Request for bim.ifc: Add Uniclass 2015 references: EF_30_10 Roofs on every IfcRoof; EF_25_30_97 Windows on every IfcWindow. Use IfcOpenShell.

First a look at what the model holds.

```python
import ifcopenshell

model = ifcopenshell.open("bim.ifc")
print(model.schema)
print("classifications:", [c.Name for c in model.by_type("IfcClassification")])
for ifc_class in ("IfcDoor", "IfcRoof", "IfcStair", "IfcWall", "IfcWindow"):
    print(ifc_class, len(model.by_type(ifc_class)))
```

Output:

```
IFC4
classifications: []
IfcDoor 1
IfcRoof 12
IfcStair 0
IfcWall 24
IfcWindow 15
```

```python
import ifcopenshell
import ifcopenshell.api.classification

model = ifcopenshell.open("bim.ifc")

system = ifcopenshell.api.classification.add_classification(model, classification="Uniclass 2015")

codes = {
    "IfcRoof": ("EF_30_10", "Roofs"),
    "IfcWindow": ("EF_25_30_97", "Windows"),
}
for ifc_class, (code, name) in codes.items():
    products = model.by_type(ifc_class)
    ifcopenshell.api.classification.add_reference(
        model, products=products, classification=system, identification=code, name=name
    )
    print(code, len(products))

model.write("bim_rev.ifc")
```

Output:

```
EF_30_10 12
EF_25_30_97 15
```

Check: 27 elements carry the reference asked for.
